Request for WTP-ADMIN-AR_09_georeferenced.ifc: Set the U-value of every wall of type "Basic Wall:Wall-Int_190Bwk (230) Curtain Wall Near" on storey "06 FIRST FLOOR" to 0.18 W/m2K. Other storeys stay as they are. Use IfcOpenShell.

First a look at what the model holds.

```python
import ifcopenshell
import ifcopenshell.util.element

model = ifcopenshell.open("WTP-ADMIN-AR_09_georeferenced.ifc")
print(model.schema)
storey = next(s for s in model.by_type("IfcBuildingStorey") if s.Name == "06 FIRST FLOOR")
walls = [e for e in ifcopenshell.util.element.get_decomposition(storey) if e.is_a("IfcWall")]
seen = {}
for e in walls:
    element_type = ifcopenshell.util.element.get_type(e)
    key = (element_type.Name if element_type != e and element_type else None, ifcopenshell.util.element.get_pset(e, "Pset_WallCommon", "ThermalTransmittance"))
    seen[key] = seen.get(key, 0) + 1
for (name, value), count in sorted(seen.items(), key=str):
    print(count, "x", name, "|", value)
```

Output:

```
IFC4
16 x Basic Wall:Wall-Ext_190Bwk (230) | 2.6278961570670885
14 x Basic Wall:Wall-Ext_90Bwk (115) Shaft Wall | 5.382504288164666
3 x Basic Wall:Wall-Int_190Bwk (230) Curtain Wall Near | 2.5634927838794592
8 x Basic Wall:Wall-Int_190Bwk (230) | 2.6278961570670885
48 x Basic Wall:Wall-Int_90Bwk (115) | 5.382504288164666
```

```python
import ifcopenshell
import ifcopenshell.api.pset
import ifcopenshell.util.element

model = ifcopenshell.open("WTP-ADMIN-AR_09_georeferenced.ifc")

storey = next(s for s in model.by_type("IfcBuildingStorey") if s.Name == "06 FIRST FLOOR")
walls = [e for e in ifcopenshell.util.element.get_decomposition(storey) if e.is_a("IfcWall")]

count = 0
for e in walls:
    element_type = ifcopenshell.util.element.get_type(e)
    if element_type in (None, e) or element_type.Name != "Basic Wall:Wall-Int_190Bwk (230) Curtain Wall Near":
        continue
    # add_pset returns the element's existing set when there is one.
    pset = ifcopenshell.api.pset.add_pset(model, product=e, name="Pset_WallCommon")
    ifcopenshell.api.pset.edit_pset(model, pset=pset, properties={"ThermalTransmittance": 0.18})
    count += 1

print(count, "walls updated")

model.write("WTP-ADMIN-AR_09_georeferenced-out.ifc")
```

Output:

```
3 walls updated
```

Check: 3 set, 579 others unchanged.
